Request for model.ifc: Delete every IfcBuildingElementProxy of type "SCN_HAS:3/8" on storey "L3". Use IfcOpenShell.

First a look at what the model holds.

```python
import ifcopenshell
import ifcopenshell.util.element

model = ifcopenshell.open("model.ifc")
print(model.schema)
storey = next(s for s in model.by_type("IfcBuildingStorey") if s.Name == "L3")
proxies = [e for e in ifcopenshell.util.element.get_decomposition(storey) if e.is_a("IfcBuildingElementProxy")]
seen = {}
for e in proxies:
    element_type = ifcopenshell.util.element.get_type(e)
    name = element_type.Name if element_type not in (None, e) else None
    seen[name] = seen.get(name, 0) + 1
for name, count in sorted(seen.items(), key=str):
    print(count, "x", name)
```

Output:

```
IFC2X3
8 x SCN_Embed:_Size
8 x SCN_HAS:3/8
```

```python
import ifcopenshell
import ifcopenshell.api.root
import ifcopenshell.util.element

model = ifcopenshell.open("model.ifc")

storey = next(s for s in model.by_type("IfcBuildingStorey") if s.Name == "L3")
proxies = [e for e in ifcopenshell.util.element.get_decomposition(storey) if e.is_a("IfcBuildingElementProxy")]
targets = [e for e in proxies if (t := ifcopenshell.util.element.get_type(e)) not in (None, e) and t.Name == "SCN_HAS:3/8"]

for e in targets:
    ifcopenshell.api.root.remove_product(model, product=e)
print(len(targets), "removed")

model.write("model-out.ifc")
```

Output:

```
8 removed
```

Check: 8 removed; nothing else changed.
